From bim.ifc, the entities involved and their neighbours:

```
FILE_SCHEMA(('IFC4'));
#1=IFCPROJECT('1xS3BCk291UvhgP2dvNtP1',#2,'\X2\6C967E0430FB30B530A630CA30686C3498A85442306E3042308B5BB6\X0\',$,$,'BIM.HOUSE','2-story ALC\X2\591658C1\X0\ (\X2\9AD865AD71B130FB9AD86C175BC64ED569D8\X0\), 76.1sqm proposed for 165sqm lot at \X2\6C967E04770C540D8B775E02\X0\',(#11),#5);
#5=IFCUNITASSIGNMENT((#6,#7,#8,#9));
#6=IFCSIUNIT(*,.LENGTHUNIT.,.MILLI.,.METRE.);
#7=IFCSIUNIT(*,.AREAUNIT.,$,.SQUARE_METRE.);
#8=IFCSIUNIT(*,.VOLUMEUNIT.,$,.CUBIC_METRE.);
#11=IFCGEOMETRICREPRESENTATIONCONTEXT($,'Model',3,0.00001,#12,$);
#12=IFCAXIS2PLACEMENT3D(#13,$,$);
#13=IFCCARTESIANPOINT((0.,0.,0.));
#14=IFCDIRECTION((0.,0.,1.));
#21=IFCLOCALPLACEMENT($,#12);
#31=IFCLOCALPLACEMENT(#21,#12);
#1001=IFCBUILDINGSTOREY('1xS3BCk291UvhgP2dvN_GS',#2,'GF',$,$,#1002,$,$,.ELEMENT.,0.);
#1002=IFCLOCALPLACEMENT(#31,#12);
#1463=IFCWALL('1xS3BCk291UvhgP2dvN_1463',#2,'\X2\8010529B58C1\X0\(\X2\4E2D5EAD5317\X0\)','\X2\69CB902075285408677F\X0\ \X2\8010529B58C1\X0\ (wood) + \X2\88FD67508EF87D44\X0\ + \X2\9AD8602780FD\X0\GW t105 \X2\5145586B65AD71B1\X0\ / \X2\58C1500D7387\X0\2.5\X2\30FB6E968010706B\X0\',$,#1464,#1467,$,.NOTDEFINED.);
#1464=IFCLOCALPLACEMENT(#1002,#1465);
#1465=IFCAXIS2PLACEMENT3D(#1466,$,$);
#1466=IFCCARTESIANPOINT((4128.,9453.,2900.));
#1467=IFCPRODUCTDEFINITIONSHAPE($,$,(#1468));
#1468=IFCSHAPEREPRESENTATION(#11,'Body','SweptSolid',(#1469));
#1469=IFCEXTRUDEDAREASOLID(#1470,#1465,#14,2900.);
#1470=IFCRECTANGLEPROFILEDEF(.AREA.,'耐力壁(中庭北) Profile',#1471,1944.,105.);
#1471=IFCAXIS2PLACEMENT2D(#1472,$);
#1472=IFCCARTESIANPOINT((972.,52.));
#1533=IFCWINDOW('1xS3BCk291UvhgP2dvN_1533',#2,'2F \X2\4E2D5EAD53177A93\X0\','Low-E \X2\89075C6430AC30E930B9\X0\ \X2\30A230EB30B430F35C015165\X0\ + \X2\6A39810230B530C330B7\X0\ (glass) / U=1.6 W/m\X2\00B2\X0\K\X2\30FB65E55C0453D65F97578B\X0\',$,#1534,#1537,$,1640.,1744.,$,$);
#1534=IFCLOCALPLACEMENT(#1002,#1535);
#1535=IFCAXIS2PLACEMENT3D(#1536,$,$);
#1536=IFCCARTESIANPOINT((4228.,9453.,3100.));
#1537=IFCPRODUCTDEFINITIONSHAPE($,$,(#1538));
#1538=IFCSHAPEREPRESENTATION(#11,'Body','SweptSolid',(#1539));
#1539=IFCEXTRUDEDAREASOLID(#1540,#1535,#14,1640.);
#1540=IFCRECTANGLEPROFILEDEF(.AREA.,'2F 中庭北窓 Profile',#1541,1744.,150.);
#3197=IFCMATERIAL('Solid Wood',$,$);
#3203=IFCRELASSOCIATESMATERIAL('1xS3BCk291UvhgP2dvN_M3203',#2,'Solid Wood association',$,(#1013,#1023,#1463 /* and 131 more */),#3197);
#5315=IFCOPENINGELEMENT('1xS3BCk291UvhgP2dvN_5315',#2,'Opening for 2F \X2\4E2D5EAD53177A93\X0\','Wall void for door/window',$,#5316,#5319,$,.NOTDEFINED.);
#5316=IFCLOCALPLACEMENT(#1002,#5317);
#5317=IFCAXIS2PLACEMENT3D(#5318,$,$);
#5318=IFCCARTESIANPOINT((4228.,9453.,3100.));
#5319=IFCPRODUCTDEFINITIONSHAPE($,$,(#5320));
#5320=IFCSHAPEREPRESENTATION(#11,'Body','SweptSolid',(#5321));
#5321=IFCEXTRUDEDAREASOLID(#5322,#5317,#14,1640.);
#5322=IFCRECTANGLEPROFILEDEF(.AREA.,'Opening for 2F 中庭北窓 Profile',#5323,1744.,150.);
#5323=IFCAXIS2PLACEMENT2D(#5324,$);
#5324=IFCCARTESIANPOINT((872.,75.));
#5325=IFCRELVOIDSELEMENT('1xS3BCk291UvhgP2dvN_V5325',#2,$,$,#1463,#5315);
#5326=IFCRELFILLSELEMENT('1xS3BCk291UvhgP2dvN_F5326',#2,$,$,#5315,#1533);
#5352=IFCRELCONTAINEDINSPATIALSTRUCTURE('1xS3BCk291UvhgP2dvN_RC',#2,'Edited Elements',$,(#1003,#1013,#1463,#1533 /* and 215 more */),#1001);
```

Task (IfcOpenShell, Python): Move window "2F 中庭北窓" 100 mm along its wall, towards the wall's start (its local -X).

```python
import ifcopenshell
import ifcopenshell.api.geometry
import ifcopenshell.util.placement

model = ifcopenshell.open("bim.ifc")

window = model.by_guid("1xS3BCk291UvhgP2dvN_1533")
opening = window.FillsVoids[0].RelatingOpeningElement
wall = opening.VoidsElements[0].RelatingBuildingElement

wall_matrix = ifcopenshell.util.placement.get_local_placement(wall.ObjectPlacement)
shift = wall_matrix[:3, 0] * -100.0
before = ifcopenshell.util.placement.get_local_placement(window.ObjectPlacement)[:3, 3].copy()

# The window is not placed relative to its opening, so move both.
for product in (opening, window):
    matrix = ifcopenshell.util.placement.get_local_placement(product.ObjectPlacement)
    matrix[:3, 3] += shift
    ifcopenshell.api.geometry.edit_object_placement(model, product=product, matrix=matrix, is_si=False)

after = ifcopenshell.util.placement.get_local_placement(window.ObjectPlacement)[:3, 3]
print("window moved by", (after - before).round(3) + 0.0)

model.write("bim_v2.ifc")
```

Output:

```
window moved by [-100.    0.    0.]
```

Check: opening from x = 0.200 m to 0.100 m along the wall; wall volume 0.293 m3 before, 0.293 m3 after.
